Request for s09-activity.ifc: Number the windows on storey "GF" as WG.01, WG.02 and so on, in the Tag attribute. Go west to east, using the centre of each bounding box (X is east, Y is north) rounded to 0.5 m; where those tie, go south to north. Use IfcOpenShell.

First a look at what the model holds.

```python
import ifcopenshell
import ifcopenshell.util.element
import ifcopenshell.util.placement

model = ifcopenshell.open("s09-activity.ifc")
print(model.schema)
storey = next(s for s in model.by_type("IfcBuildingStorey") if s.Name == "GF")
windows = [e for e in ifcopenshell.util.element.get_decomposition(storey) if e.is_a("IfcWindow")]
for e in sorted(windows, key=lambda e: e.id()):
    origin = ifcopenshell.util.placement.get_local_placement(e.ObjectPlacement)[:3, 3]
    print(e.id(), e.Tag, e.Name, origin.round(2) + 0.0, sep=" | ")
```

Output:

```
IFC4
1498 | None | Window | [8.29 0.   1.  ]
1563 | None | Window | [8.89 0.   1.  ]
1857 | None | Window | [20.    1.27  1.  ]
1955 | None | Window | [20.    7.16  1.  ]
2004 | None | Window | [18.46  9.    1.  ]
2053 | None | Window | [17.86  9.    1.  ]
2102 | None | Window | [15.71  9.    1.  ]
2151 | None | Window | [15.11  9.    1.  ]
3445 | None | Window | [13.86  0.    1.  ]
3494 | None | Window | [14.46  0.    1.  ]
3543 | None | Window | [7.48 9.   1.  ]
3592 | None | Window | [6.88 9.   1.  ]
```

```python
import ifcopenshell
import ifcopenshell.geom
import ifcopenshell.util.element
import ifcopenshell.util.shape

model = ifcopenshell.open("s09-activity.ifc")
settings = ifcopenshell.geom.settings()
settings.set("use-world-coords", True)


def centre(element):
    shape = ifcopenshell.geom.create_shape(settings, element)
    return ifcopenshell.util.shape.get_bbox_centroid(shape.geometry)


storey = next(s for s in model.by_type("IfcBuildingStorey") if s.Name == "GF")
windows = [e for e in ifcopenshell.util.element.get_decomposition(storey) if e.is_a("IfcWindow")]

# Insertion points can sit at a corner or the storey origin, so sort by the geometry (in metres).
centres = {e: centre(e) for e in windows}
windows.sort(key=lambda e: (round(centres[e][0] / 0.5), centres[e][1]))

for i, e in enumerate(windows, start=1):
    number = f"WG.{i:02d}"
    e.Tag = number
    print(e.id(), number)

model.write("s09-activity_rev.ifc")
```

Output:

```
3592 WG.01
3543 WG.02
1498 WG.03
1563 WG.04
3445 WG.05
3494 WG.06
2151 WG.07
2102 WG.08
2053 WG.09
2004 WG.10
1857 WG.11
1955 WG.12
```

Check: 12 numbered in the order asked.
